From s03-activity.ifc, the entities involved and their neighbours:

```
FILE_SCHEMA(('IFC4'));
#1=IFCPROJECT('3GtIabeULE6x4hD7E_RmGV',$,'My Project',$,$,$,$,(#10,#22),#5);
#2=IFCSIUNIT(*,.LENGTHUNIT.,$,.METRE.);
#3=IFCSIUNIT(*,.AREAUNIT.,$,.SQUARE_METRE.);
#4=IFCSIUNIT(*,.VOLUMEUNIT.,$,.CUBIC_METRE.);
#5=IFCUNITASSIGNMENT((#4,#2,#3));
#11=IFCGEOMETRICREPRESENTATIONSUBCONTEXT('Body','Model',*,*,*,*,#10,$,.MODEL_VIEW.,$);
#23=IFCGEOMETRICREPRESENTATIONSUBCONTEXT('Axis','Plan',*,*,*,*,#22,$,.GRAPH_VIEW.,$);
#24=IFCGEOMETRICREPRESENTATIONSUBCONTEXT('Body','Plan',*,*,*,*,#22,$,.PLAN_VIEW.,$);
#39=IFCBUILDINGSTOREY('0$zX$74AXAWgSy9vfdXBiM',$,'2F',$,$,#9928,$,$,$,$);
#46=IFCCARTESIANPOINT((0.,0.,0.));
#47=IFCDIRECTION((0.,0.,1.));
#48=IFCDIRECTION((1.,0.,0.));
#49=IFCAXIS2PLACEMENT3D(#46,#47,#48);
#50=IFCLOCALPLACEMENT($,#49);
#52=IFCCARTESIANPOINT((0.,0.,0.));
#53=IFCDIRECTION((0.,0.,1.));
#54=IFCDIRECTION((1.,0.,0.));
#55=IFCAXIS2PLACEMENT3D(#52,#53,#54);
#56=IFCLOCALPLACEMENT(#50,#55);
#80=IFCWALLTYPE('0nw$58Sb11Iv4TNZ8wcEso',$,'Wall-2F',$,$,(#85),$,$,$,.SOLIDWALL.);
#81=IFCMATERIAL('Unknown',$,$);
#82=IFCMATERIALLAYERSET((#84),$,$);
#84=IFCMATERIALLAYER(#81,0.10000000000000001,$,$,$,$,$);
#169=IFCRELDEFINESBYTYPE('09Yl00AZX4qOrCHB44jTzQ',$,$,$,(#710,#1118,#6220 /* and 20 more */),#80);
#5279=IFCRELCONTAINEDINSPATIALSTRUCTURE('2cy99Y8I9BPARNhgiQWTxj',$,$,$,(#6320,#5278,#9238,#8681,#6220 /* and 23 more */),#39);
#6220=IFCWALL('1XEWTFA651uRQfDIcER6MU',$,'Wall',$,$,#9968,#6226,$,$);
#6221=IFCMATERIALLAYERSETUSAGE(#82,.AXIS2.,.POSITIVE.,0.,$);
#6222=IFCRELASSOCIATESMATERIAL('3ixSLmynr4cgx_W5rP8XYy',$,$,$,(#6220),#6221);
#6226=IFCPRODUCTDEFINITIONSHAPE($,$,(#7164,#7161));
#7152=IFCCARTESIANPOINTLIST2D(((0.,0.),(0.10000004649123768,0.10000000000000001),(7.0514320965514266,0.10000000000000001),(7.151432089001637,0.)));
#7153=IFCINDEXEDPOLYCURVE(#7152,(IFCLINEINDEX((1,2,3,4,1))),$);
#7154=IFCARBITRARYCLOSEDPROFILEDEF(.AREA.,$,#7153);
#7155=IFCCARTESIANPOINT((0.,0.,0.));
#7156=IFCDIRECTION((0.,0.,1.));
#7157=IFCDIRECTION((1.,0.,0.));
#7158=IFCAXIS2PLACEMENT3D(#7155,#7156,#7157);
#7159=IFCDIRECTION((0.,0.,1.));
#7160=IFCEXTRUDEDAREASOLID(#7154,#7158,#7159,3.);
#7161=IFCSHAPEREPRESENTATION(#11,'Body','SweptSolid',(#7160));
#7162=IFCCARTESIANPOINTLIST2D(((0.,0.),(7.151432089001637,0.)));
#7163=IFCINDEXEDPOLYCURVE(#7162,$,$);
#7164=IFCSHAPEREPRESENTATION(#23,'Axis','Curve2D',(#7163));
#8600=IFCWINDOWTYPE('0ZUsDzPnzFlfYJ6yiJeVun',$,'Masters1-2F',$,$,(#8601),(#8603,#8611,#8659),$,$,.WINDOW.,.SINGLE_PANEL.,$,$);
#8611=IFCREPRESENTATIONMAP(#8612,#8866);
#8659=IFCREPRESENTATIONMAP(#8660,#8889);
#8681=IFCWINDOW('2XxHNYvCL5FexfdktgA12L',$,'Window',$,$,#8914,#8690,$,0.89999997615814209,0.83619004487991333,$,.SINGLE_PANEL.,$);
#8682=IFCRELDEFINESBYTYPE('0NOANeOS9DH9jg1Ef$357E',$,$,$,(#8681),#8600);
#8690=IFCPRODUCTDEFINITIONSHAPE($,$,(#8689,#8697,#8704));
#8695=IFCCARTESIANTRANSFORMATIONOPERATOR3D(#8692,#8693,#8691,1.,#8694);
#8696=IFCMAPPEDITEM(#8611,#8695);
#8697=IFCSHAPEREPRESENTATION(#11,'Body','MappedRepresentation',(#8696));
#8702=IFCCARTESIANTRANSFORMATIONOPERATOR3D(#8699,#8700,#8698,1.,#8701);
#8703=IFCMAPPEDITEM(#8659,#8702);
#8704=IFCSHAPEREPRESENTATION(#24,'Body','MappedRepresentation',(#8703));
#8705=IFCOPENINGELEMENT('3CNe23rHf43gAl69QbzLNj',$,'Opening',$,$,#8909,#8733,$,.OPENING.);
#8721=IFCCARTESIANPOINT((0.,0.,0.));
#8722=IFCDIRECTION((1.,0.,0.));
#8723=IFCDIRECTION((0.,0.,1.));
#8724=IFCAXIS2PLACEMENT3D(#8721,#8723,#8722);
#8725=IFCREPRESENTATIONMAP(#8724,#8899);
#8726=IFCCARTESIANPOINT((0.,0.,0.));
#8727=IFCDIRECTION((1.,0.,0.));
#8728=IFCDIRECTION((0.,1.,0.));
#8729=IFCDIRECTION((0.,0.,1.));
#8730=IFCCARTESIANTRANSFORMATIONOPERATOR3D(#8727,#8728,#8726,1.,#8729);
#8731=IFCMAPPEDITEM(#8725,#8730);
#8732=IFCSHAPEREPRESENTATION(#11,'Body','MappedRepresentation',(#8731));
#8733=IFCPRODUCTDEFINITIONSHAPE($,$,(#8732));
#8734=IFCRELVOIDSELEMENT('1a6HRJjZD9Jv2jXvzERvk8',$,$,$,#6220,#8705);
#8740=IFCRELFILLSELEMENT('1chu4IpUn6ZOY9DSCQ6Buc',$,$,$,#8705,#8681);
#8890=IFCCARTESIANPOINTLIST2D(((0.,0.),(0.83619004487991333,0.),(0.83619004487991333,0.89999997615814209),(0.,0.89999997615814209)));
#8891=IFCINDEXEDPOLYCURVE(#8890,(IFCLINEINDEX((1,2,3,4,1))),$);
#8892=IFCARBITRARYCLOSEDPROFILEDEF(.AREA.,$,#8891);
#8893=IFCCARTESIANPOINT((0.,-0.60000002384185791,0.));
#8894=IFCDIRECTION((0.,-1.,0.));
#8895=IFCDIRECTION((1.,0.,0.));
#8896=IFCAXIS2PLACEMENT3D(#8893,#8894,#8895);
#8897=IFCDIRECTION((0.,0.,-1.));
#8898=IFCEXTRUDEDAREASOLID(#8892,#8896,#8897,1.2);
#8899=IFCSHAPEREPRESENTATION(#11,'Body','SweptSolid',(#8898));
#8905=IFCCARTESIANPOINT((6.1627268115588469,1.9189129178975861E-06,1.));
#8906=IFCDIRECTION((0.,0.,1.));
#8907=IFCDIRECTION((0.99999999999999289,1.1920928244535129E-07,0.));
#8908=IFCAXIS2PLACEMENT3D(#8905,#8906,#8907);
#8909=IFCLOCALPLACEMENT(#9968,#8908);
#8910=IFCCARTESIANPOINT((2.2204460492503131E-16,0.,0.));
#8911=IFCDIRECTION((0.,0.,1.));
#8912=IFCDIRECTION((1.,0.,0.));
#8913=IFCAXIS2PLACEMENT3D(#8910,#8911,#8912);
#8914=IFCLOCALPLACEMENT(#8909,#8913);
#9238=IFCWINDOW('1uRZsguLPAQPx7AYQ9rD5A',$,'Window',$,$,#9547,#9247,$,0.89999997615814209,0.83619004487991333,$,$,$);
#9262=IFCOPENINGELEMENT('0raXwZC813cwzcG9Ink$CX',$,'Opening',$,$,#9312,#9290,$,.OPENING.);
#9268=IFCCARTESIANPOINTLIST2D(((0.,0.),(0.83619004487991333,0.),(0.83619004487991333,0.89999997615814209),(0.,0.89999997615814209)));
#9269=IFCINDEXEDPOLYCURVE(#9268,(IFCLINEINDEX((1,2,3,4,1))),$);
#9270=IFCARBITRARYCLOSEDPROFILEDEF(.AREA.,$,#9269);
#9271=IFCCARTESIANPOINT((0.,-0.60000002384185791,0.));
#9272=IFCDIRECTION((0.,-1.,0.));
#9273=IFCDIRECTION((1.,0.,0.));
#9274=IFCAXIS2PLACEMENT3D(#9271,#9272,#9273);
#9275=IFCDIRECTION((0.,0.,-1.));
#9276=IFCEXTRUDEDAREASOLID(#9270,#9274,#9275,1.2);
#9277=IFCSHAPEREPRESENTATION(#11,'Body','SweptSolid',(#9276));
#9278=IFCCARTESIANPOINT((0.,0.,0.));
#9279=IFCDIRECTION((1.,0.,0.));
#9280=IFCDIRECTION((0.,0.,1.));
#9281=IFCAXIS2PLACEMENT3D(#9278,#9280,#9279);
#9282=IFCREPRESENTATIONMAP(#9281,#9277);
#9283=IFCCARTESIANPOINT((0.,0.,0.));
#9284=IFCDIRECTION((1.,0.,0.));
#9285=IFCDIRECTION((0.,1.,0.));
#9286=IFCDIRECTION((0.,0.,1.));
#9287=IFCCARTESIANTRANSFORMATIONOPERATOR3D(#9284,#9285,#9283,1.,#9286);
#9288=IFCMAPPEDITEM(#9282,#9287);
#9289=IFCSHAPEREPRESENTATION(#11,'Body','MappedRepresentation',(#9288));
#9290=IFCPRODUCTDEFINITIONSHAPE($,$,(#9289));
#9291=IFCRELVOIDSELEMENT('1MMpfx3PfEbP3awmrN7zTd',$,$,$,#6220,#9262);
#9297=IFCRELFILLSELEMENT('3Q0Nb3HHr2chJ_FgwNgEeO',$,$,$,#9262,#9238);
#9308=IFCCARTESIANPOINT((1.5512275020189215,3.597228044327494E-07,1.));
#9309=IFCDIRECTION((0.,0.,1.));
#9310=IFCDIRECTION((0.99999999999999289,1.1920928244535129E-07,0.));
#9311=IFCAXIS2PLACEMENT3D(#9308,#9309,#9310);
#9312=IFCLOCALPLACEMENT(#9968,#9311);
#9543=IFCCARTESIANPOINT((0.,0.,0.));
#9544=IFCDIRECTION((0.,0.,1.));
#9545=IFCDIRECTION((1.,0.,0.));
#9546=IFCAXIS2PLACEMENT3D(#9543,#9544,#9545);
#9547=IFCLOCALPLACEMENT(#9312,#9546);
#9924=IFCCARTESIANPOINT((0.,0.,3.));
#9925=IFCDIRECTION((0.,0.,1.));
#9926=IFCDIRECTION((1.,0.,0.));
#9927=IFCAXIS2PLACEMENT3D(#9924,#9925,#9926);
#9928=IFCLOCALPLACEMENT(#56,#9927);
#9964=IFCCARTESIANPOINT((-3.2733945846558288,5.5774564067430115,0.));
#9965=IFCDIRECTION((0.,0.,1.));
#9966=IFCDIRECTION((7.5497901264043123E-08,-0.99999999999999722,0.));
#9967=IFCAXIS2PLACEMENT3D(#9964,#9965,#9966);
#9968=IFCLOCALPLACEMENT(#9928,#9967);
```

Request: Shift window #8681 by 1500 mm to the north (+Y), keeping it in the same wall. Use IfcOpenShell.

```python
import ifcopenshell
import ifcopenshell.api.geometry
import ifcopenshell.util.placement
import ifcopenshell.util.unit

model = ifcopenshell.open("s03-activity.ifc")
unit_scale = ifcopenshell.util.unit.calculate_unit_scale(model)

window = model.by_guid("2XxHNYvCL5FexfdktgA12L")
opening = window.FillsVoids[0].RelatingOpeningElement
wall = opening.VoidsElements[0].RelatingBuildingElement

wall_matrix = ifcopenshell.util.placement.get_local_placement(wall.ObjectPlacement)
shift = wall_matrix[:3, 0] * -1.5 / unit_scale
before = ifcopenshell.util.placement.get_local_placement(window.ObjectPlacement)[:3, 3].copy()

# The window is placed relative to its opening, so it follows when the opening moves.
matrix = ifcopenshell.util.placement.get_local_placement(opening.ObjectPlacement)
matrix[:3, 3] += shift
ifcopenshell.api.geometry.edit_object_placement(
    model, product=opening, matrix=matrix, is_si=False, should_transform_children=True
)

after = ifcopenshell.util.placement.get_local_placement(window.ObjectPlacement)[:3, 3]
print("window moved by", (after - before).round(3) + 0.0)

model.write("s03-activity_updated.ifc")
```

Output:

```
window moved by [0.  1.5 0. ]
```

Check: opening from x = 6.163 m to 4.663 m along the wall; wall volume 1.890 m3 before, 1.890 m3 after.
